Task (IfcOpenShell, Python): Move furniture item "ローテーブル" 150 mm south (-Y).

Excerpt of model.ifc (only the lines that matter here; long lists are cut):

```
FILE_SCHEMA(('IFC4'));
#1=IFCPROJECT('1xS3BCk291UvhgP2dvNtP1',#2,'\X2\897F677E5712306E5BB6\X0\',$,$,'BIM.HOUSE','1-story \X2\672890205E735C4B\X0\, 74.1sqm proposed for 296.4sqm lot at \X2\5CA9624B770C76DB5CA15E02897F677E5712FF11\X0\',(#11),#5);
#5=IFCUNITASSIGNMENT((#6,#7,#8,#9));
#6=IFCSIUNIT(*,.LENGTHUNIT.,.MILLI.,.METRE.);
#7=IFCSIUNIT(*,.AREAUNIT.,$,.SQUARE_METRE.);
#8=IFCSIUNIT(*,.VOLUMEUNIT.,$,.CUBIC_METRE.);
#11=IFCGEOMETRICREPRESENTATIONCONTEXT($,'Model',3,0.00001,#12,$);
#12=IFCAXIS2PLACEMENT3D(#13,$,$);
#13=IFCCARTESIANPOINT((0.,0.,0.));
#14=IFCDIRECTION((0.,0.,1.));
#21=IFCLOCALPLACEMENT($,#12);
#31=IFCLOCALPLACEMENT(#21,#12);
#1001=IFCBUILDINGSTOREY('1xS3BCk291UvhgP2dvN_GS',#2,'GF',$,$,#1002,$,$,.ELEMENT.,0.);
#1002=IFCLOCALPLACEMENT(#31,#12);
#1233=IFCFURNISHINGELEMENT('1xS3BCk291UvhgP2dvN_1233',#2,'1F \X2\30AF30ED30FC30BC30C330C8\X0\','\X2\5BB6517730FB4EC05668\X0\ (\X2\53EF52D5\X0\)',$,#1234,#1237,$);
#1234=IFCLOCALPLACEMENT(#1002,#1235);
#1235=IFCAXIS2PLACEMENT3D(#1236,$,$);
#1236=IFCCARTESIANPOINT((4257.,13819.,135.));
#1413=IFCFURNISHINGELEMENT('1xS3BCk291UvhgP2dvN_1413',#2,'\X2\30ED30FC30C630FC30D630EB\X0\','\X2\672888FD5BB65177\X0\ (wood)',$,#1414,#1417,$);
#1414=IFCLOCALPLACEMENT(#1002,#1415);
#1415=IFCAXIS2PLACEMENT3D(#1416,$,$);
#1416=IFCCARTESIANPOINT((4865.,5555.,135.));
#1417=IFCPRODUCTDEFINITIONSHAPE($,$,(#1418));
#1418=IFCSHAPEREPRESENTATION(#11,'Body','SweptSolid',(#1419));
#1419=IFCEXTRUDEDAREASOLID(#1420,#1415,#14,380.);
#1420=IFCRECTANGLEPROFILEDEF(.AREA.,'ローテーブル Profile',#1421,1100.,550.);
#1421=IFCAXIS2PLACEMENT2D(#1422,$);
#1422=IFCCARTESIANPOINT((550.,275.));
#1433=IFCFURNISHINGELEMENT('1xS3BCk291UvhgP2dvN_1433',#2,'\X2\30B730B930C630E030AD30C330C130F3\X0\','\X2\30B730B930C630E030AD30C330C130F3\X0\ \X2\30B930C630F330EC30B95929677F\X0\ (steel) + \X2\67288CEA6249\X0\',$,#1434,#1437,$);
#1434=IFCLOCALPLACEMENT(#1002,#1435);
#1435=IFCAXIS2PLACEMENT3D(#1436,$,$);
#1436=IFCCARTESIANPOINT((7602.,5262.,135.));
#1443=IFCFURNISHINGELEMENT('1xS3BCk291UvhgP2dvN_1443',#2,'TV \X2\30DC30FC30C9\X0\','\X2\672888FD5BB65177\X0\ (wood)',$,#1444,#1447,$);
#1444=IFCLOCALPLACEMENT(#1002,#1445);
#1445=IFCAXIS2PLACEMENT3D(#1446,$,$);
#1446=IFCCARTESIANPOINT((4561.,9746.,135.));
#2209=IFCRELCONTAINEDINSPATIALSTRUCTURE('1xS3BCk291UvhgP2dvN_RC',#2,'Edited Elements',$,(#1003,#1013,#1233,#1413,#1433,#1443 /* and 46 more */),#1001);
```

```python
import ifcopenshell
import ifcopenshell.api.geometry
import ifcopenshell.util.placement
import ifcopenshell.util.unit

model = ifcopenshell.open("model.ifc")
unit_scale = ifcopenshell.util.unit.calculate_unit_scale(model)

item = model.by_id(1413)
matrix = ifcopenshell.util.placement.get_local_placement(item.ObjectPlacement)
matrix[1, 3] -= 0.15 / unit_scale
ifcopenshell.api.geometry.edit_object_placement(model, product=item, matrix=matrix, is_si=False)

print(ifcopenshell.util.placement.get_local_placement(item.ObjectPlacement).round(3) + 0.0)

model.write("model_updated.ifc")
```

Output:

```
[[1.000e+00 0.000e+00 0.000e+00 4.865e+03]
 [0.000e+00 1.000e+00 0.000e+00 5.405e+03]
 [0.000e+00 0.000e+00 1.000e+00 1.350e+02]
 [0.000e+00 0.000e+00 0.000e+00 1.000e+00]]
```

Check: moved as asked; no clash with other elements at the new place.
